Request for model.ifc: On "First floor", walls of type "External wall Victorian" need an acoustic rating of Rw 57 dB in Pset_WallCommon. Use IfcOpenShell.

First a look at what the model holds.

```python
import ifcopenshell
import ifcopenshell.util.element

model = ifcopenshell.open("model.ifc")
print(model.schema)
storey = next(s for s in model.by_type("IfcBuildingStorey") if s.Name == "First floor")
walls = [e for e in ifcopenshell.util.element.get_decomposition(storey) if e.is_a("IfcWall")]
seen = {}
for e in walls:
    element_type = ifcopenshell.util.element.get_type(e)
    key = (element_type.Name if element_type != e and element_type else None, ifcopenshell.util.element.get_pset(e, "Pset_WallCommon", "AcousticRating"))
    seen[key] = seen.get(key, 0) + 1
for (name, value), count in sorted(seen.items(), key=str):
    print(count, "x", name, "|", value)
```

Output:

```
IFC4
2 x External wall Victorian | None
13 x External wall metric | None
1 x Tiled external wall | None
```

```python
import ifcopenshell
import ifcopenshell.api.pset
import ifcopenshell.util.element

model = ifcopenshell.open("model.ifc")

storey = next(s for s in model.by_type("IfcBuildingStorey") if s.Name == "First floor")
walls = [e for e in ifcopenshell.util.element.get_decomposition(storey) if e.is_a("IfcWall")]

count = 0
for e in walls:
    element_type = ifcopenshell.util.element.get_type(e)
    if element_type in (None, e) or element_type.Name != "External wall Victorian":
        continue
    # add_pset returns the element's existing set when there is one.
    pset = ifcopenshell.api.pset.add_pset(model, product=e, name="Pset_WallCommon")
    ifcopenshell.api.pset.edit_pset(model, pset=pset, properties={"AcousticRating": "Rw 57 dB"})
    count += 1

print(count, "walls updated")

model.write("model_rev.ifc")
```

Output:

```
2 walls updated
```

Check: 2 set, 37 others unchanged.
